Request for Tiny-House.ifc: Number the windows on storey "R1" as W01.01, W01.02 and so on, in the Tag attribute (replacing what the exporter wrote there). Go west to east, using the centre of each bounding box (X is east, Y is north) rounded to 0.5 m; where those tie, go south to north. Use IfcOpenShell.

First a look at what the model holds.

```python
import ifcopenshell
import ifcopenshell.util.element
import ifcopenshell.util.placement

model = ifcopenshell.open("Tiny-House.ifc")
print(model.schema)
storey = next(s for s in model.by_type("IfcBuildingStorey") if s.Name == "R1")
windows = [e for e in ifcopenshell.util.element.get_decomposition(storey) if e.is_a("IfcWindow")]
for e in sorted(windows, key=lambda e: e.id()):
    origin = ifcopenshell.util.placement.get_local_placement(e.ObjectPlacement)[:3, 3]
    print(e.id(), e.Tag, e.Name, origin.round(2) + 0.0, sep=" | ")
```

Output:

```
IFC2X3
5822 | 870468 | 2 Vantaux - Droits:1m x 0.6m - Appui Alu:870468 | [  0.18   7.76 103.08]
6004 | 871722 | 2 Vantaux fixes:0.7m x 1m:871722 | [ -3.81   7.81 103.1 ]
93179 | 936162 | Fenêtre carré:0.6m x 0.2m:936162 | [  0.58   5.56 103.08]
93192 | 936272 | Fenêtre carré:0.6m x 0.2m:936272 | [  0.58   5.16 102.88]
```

```python
import ifcopenshell
import ifcopenshell.geom
import ifcopenshell.util.element
import ifcopenshell.util.shape

model = ifcopenshell.open("Tiny-House.ifc")
settings = ifcopenshell.geom.settings()
settings.set("use-world-coords", True)


def centre(element):
    shape = ifcopenshell.geom.create_shape(settings, element)
    return ifcopenshell.util.shape.get_bbox_centroid(shape.geometry)


storey = next(s for s in model.by_type("IfcBuildingStorey") if s.Name == "R1")
windows = [e for e in ifcopenshell.util.element.get_decomposition(storey) if e.is_a("IfcWindow")]

# Insertion points can sit at a corner or the storey origin, so sort by the geometry (in metres).
centres = {e: centre(e) for e in windows}
windows.sort(key=lambda e: (round(centres[e][0] / 0.5), centres[e][1]))

for i, e in enumerate(windows, start=1):
    number = f"W01.{i:02d}"
    e.Tag = number
    print(e.id(), number)

model.write("Tiny-House_rev.ifc")
```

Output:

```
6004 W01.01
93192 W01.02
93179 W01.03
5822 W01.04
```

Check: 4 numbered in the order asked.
